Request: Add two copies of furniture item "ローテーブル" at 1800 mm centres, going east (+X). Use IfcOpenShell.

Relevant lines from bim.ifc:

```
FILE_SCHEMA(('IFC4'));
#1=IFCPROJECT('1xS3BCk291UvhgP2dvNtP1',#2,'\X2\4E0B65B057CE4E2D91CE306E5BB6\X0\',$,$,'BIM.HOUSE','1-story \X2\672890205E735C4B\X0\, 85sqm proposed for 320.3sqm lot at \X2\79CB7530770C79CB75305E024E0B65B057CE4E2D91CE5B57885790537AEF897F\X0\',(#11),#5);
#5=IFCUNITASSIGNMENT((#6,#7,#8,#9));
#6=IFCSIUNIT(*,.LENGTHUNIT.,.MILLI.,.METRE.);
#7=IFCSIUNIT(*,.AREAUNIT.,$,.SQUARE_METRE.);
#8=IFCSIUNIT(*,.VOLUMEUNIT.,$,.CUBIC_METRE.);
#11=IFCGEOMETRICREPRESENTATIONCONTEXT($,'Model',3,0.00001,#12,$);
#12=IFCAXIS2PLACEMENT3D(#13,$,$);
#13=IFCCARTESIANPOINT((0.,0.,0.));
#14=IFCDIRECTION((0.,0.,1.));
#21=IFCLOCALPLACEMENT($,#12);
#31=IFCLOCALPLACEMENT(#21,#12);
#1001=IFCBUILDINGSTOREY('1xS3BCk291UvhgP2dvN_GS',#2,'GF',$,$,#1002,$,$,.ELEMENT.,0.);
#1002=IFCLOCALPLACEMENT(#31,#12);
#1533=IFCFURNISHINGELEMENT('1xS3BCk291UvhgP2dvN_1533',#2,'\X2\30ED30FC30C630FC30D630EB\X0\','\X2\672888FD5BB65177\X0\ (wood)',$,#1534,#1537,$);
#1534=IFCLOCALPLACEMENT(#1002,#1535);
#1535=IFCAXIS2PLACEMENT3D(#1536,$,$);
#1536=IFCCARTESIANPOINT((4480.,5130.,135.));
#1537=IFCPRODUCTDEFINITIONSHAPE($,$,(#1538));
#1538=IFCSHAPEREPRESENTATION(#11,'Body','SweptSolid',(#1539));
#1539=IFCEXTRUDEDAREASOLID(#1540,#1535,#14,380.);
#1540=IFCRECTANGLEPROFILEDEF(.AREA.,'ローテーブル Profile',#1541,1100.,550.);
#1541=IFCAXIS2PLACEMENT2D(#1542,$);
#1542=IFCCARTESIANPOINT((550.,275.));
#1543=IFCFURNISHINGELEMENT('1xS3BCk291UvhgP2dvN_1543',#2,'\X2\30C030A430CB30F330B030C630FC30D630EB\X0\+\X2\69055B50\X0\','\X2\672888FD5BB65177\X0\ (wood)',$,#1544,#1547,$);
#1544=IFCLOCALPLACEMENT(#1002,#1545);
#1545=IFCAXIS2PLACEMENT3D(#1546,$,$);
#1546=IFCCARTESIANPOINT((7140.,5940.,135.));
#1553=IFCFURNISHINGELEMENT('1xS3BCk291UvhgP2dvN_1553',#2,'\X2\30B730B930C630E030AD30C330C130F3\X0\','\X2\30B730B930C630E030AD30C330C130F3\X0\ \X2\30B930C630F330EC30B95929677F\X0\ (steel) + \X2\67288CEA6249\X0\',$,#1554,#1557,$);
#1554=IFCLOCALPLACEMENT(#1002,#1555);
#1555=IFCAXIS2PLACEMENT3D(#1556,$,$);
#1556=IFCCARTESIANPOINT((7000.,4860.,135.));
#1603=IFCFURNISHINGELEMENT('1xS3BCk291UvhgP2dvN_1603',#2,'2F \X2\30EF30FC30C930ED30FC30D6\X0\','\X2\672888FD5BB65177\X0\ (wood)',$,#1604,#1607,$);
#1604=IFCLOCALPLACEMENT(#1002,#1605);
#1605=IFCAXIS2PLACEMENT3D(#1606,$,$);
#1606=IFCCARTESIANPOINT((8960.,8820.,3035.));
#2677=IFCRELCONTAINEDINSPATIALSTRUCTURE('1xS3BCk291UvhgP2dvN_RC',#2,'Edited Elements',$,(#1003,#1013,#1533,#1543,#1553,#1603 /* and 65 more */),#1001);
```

```python
import numpy as np
import ifcopenshell
import ifcopenshell.api.geometry
import ifcopenshell.api.root
import ifcopenshell.util.element
import ifcopenshell.util.placement

model = ifcopenshell.open("bim.ifc")


def reuse_history(source, copy):
    """copy_class also copies each property set's owner history, people and application; keep the originals."""
    for rel in copy.IsDefinedBy:
        if rel.is_a("IfcRelDefinesByProperties") and (history := rel.RelatingPropertyDefinition.OwnerHistory):
            rel.RelatingPropertyDefinition.OwnerHistory = source.OwnerHistory
            ifcopenshell.util.element.remove_deep2(model, history)


source = model.by_guid("1xS3BCk291UvhgP2dvN_1533")
base = ifcopenshell.util.placement.get_local_placement(source.ObjectPlacement)
step = np.array([1.0, 0.0, 0.0]) * 1800.0

for i in range(1, 3):
    copy = ifcopenshell.api.root.copy_class(model, product=source)
    copy.Representation = ifcopenshell.util.element.copy_deep(
        model, source.Representation, exclude=["IfcGeometricRepresentationContext", "IfcRepresentationMap"]
    )
    reuse_history(source, copy)
    matrix = base.copy()
    matrix[:3, 3] += i * step
    print("added at", matrix[:3, 3].round(3) + 0.0)
    ifcopenshell.api.geometry.edit_object_placement(model, product=copy, matrix=matrix, is_si=False)

model.write("bim_updated.ifc")
```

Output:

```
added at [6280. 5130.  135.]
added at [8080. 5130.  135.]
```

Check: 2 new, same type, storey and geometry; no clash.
